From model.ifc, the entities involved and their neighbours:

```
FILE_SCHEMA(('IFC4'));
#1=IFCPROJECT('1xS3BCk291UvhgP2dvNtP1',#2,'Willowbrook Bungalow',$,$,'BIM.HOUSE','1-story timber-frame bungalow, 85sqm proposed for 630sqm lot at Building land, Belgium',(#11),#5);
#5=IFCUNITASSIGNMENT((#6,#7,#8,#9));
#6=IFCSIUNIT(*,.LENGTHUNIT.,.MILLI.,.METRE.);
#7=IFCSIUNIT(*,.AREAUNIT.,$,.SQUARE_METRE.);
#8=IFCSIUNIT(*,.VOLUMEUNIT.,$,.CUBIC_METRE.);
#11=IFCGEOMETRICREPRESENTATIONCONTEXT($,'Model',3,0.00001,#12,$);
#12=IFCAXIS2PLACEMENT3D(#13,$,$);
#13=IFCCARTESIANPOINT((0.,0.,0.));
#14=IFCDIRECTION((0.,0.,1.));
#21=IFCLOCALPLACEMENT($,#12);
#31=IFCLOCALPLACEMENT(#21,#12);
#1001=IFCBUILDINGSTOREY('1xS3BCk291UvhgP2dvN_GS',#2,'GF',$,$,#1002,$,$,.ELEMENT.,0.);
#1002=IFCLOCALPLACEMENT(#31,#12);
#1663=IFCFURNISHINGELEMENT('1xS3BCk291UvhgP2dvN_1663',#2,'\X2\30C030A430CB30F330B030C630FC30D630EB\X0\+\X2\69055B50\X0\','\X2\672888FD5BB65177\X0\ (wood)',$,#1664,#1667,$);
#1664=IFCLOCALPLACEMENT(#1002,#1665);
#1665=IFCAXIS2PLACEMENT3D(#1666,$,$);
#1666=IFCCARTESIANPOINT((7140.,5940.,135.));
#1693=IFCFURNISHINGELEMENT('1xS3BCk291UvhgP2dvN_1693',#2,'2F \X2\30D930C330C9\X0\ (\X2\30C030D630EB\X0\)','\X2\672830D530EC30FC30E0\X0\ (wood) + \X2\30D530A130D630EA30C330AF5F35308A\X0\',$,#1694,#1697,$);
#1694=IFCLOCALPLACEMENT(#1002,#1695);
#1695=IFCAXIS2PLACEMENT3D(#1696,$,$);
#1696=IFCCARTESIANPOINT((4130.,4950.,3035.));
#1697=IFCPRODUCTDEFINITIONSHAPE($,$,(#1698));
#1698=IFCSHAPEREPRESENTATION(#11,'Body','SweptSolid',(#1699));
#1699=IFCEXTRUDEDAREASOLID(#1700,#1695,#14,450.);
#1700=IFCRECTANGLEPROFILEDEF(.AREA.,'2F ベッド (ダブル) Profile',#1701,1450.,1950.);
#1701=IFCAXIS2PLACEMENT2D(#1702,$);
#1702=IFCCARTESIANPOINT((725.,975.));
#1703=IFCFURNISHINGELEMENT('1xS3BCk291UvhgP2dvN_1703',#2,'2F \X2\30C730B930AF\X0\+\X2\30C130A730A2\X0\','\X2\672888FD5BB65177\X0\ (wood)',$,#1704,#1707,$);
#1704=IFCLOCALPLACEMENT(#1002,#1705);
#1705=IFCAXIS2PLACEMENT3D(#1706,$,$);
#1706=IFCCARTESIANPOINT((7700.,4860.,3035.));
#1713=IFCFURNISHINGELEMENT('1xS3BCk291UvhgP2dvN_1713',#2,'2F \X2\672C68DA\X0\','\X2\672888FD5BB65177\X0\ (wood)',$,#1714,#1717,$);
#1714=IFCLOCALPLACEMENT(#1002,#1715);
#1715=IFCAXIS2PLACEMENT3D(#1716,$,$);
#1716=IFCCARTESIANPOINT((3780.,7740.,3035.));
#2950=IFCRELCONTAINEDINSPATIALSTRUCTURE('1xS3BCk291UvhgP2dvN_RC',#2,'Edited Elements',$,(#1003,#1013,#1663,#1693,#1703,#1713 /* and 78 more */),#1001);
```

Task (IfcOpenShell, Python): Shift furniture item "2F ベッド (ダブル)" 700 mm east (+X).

```python
import ifcopenshell
import ifcopenshell.api.geometry
import ifcopenshell.util.placement

model = ifcopenshell.open("model.ifc")

item = model.by_id(1693)
matrix = ifcopenshell.util.placement.get_local_placement(item.ObjectPlacement)
matrix[0, 3] += 700.0
ifcopenshell.api.geometry.edit_object_placement(model, product=item, matrix=matrix, is_si=False)

print(ifcopenshell.util.placement.get_local_placement(item.ObjectPlacement).round(3) + 0.0)

model.write("model-out.ifc")
```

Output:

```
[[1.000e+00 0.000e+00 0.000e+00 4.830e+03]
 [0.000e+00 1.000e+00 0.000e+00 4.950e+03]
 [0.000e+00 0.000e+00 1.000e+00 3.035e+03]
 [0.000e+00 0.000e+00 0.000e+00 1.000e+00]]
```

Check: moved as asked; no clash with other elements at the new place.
